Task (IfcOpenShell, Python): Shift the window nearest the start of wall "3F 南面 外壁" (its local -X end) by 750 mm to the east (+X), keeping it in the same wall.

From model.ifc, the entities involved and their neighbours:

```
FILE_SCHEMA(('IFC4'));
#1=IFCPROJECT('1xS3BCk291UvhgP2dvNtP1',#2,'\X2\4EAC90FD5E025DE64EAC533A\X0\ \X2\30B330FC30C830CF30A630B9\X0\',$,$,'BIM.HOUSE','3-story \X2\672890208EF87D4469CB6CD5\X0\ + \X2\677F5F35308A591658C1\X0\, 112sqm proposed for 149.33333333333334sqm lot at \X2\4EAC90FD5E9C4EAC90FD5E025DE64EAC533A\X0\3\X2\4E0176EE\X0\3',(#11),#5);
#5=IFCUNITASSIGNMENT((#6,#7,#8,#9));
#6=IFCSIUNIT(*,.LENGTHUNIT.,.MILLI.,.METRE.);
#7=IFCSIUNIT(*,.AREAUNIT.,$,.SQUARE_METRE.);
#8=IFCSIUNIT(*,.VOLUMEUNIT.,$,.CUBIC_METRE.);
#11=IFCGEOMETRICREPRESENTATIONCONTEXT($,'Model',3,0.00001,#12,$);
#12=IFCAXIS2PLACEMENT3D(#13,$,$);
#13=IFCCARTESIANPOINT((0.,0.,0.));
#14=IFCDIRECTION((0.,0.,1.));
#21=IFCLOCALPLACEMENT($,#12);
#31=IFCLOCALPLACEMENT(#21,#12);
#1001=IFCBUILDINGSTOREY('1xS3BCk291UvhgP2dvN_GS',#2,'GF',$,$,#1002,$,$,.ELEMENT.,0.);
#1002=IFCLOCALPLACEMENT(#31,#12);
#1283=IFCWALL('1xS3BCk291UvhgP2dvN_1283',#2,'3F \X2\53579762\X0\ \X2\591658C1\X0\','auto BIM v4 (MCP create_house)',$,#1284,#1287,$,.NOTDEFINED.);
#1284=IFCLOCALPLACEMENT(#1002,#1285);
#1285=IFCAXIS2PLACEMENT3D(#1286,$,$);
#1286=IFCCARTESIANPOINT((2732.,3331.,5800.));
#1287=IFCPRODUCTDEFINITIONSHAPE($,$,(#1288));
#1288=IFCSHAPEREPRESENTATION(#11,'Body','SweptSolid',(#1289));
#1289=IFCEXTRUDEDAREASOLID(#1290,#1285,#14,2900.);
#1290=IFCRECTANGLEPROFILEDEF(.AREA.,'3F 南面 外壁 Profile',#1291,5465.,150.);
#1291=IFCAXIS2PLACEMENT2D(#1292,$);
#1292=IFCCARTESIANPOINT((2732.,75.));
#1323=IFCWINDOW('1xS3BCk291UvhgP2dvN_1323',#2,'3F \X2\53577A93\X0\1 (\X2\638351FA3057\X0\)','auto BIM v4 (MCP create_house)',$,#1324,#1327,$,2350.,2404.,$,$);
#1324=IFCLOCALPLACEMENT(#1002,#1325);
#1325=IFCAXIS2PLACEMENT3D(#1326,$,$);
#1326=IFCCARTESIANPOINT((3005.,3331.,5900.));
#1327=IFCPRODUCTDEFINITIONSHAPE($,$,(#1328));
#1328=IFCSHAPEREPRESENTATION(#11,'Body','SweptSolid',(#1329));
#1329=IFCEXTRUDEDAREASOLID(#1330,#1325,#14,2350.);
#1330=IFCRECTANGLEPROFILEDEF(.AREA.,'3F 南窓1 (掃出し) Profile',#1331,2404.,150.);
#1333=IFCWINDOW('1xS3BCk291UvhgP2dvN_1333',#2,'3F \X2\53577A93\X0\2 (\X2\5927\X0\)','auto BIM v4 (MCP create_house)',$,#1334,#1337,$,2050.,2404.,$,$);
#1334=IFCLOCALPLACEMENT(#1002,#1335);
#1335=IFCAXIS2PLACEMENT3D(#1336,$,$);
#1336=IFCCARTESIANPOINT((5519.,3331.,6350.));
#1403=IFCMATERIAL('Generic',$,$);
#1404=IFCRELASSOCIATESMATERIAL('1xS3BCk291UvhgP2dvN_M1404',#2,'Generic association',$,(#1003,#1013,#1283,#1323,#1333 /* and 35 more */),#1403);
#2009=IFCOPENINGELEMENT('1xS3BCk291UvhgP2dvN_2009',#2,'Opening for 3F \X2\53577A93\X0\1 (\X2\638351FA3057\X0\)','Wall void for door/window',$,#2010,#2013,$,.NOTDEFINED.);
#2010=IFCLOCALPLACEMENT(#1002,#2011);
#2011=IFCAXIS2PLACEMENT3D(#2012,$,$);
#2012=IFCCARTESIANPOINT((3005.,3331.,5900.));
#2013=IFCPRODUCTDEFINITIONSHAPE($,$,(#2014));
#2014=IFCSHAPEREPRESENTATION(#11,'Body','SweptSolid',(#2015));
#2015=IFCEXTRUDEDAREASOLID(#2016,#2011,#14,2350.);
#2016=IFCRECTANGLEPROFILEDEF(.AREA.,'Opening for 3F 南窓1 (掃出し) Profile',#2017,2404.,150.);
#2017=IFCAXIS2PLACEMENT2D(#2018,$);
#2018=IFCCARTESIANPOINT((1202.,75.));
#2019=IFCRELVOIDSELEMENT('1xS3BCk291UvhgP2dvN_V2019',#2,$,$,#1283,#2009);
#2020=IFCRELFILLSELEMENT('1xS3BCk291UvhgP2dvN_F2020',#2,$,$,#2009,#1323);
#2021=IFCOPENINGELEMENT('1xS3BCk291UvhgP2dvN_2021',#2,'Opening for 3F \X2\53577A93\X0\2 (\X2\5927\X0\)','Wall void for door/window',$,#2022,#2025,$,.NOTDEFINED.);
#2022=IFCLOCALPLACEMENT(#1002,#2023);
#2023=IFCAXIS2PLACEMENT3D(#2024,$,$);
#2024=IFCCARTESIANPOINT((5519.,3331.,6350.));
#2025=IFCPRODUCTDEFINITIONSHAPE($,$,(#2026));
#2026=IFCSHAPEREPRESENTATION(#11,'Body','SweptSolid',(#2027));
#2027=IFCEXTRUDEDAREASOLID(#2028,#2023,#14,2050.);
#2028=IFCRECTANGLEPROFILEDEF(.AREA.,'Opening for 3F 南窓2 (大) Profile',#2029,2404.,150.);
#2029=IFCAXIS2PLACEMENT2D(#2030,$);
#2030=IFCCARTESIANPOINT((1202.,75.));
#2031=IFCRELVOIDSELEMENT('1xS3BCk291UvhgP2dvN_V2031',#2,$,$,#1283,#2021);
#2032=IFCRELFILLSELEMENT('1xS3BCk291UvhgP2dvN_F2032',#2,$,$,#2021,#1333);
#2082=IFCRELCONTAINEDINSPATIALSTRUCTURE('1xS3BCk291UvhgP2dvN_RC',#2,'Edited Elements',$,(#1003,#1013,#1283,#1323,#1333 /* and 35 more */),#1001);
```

```python
import ifcopenshell
import ifcopenshell.api.geometry
import ifcopenshell.util.placement
import ifcopenshell.util.unit

model = ifcopenshell.open("model.ifc")
unit_scale = ifcopenshell.util.unit.calculate_unit_scale(model)

window = model.by_guid("1xS3BCk291UvhgP2dvN_1323")
opening = window.FillsVoids[0].RelatingOpeningElement
wall = opening.VoidsElements[0].RelatingBuildingElement

wall_matrix = ifcopenshell.util.placement.get_local_placement(wall.ObjectPlacement)
shift = wall_matrix[:3, 0] * 0.75 / unit_scale
before = ifcopenshell.util.placement.get_local_placement(window.ObjectPlacement)[:3, 3].copy()

# The window is not placed relative to its opening, so move both.
for product in (opening, window):
    matrix = ifcopenshell.util.placement.get_local_placement(product.ObjectPlacement)
    matrix[:3, 3] += shift
    ifcopenshell.api.geometry.edit_object_placement(model, product=product, matrix=matrix, is_si=False)

after = ifcopenshell.util.placement.get_local_placement(window.ObjectPlacement)[:3, 3]
print("window moved by", (after - before).round(3) + 0.0)

model.write("model_v2.ifc")
```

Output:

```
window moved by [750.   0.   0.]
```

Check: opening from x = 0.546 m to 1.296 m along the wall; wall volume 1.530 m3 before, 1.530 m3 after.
